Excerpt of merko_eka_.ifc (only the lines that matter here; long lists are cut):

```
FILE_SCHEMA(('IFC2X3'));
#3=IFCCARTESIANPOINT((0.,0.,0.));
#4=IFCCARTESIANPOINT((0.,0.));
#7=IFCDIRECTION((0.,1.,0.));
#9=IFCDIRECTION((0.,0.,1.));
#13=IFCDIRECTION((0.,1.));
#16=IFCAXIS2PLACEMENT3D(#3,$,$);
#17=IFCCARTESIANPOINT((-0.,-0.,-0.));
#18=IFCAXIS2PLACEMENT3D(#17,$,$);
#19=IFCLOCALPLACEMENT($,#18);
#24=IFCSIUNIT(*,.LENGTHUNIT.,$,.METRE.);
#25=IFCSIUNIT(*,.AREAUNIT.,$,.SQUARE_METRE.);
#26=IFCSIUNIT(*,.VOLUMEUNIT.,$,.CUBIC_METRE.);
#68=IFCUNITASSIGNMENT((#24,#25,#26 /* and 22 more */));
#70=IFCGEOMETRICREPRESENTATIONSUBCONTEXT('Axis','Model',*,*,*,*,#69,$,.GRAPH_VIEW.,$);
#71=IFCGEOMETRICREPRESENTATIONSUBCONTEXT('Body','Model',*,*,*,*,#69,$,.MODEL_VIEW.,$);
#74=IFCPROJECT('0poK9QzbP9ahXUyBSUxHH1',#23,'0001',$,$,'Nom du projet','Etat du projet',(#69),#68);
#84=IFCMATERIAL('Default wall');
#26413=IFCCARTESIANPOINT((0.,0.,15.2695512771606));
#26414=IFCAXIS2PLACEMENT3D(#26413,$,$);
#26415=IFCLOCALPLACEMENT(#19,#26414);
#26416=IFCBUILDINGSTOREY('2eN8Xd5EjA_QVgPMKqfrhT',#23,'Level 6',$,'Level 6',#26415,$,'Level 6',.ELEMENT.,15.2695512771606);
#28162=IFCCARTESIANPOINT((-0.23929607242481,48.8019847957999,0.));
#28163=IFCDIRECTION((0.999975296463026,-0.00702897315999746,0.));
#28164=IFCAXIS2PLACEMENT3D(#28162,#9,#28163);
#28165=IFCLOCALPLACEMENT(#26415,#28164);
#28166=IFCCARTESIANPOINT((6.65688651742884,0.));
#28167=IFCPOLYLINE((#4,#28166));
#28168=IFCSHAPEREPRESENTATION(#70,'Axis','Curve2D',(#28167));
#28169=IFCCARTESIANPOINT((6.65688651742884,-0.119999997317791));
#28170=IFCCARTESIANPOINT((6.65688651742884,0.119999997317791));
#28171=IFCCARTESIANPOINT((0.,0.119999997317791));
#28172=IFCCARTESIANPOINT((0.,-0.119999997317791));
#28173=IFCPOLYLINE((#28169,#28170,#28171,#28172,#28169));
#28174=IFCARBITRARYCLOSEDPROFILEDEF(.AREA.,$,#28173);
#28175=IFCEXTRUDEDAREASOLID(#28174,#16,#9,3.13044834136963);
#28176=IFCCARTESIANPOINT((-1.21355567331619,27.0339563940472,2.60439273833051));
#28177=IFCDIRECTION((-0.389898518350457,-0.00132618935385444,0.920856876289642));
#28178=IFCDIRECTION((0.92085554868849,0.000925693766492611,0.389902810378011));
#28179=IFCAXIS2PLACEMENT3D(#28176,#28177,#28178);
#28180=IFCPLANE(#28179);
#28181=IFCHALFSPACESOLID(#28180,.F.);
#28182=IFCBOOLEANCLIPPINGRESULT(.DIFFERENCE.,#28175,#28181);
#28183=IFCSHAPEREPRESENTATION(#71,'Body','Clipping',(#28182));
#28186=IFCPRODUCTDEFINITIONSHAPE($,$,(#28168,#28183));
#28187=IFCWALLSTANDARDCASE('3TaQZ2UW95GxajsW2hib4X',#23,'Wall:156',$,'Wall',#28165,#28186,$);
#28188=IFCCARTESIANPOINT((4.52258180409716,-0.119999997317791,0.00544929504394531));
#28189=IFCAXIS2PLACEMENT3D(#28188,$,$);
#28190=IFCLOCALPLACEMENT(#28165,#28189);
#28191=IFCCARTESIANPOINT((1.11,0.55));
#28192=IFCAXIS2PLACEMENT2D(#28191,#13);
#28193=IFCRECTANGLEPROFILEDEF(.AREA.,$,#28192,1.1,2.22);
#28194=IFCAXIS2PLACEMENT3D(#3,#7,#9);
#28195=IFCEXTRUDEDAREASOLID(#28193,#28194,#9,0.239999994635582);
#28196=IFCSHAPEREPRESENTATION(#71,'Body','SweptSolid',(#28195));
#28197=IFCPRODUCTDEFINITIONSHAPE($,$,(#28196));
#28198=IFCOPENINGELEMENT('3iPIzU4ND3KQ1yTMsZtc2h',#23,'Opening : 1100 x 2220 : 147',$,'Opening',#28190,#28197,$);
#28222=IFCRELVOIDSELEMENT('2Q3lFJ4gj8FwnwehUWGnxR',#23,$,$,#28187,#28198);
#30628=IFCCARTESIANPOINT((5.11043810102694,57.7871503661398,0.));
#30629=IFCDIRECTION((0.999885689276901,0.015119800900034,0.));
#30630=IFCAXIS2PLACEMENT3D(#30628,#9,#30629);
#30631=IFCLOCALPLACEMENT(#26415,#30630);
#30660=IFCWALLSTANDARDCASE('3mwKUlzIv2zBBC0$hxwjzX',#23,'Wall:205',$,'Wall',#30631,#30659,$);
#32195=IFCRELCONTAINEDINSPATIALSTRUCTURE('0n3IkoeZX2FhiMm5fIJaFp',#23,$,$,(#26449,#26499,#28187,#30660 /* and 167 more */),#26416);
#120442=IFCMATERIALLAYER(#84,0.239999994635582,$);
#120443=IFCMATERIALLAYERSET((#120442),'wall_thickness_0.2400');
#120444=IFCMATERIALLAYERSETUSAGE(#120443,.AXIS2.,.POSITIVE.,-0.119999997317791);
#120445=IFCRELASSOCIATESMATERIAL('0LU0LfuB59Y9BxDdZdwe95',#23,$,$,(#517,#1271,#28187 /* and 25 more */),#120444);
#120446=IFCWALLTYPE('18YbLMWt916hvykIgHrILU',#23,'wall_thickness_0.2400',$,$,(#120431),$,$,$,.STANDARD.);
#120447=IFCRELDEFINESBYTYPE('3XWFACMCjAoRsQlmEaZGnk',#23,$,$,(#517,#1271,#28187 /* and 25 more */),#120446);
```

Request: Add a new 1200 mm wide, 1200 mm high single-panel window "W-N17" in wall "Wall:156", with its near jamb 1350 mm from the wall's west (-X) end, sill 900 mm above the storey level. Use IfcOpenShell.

```python
import numpy as np
import ifcopenshell
import ifcopenshell.api.feature
import ifcopenshell.api.geometry
import ifcopenshell.api.root
import ifcopenshell.api.spatial
import ifcopenshell.api.type
import ifcopenshell.geom
import ifcopenshell.util.element
import ifcopenshell.util.placement
import ifcopenshell.util.representation
import ifcopenshell.util.shape
import ifcopenshell.util.unit

model = ifcopenshell.open("merko_eka_.ifc")
unit_scale = ifcopenshell.util.unit.calculate_unit_scale(model)
settings = ifcopenshell.geom.settings()


def volume(element):
    """Net volume in cubic metres, openings subtracted."""
    shape = ifcopenshell.geom.create_shape(settings, element)
    return ifcopenshell.util.shape.get_volume(shape.geometry)


wall = model.by_guid("3TaQZ2UW95GxajsW2hib4X")
storey = ifcopenshell.util.element.get_container(wall, ifc_class="IfcBuildingStorey")
context = ifcopenshell.util.representation.get_context(model, "Model", "Body", "MODEL_VIEW")
before = volume(wall)

width, height, from_end, sill = 1.2, 1.2, 1.35, 0.9  # metres

# The wall runs along its own X axis, and the end named is its -X end.
wall_shape = ifcopenshell.geom.create_shape(settings, wall)
x, y, z = ifcopenshell.util.shape.get_vertices(wall_shape.geometry).T
start = x.min() + from_end
face, thickness = float(y.min()), float(y.max() - y.min())
wall_matrix = ifcopenshell.util.placement.get_local_placement(wall.ObjectPlacement)
level = ifcopenshell.util.placement.get_local_placement(storey.ObjectPlacement)[2, 3]


def in_wall(x, y):
    """Placement at x, y metres in the wall's axes, at sill height."""
    matrix = wall_matrix.copy()
    matrix[:, 3] = wall_matrix @ np.array([x / unit_scale, y / unit_scale, 0.0, 1.0])
    matrix[2, 3] = level + sill / unit_scale
    return matrix


# Opening: a box that overshoots both wall faces by 50 mm.
opening = ifcopenshell.api.root.create_entity(model, ifc_class="IfcOpeningElement")
box = ifcopenshell.api.geometry.add_wall_representation(
    model, context=context, length=width, height=height, thickness=thickness + 0.1
)
ifcopenshell.api.geometry.assign_representation(model, product=opening, representation=box)
ifcopenshell.api.geometry.edit_object_placement(model, product=opening, matrix=in_wall(start, face - 0.05), is_si=False)
ifcopenshell.api.feature.add_feature(model, feature=opening, element=wall)

window = ifcopenshell.api.root.create_entity(model, ifc_class="IfcWindow", name="W-N17")
window.OverallWidth, window.OverallHeight = width / unit_scale, height / unit_scale
body = ifcopenshell.api.geometry.add_window_representation(
    model,
    context=context,
    overall_width=window.OverallWidth,
    overall_height=window.OverallHeight,
    partition_type="SINGLE_PANEL",
)
ifcopenshell.api.geometry.assign_representation(model, product=window, representation=body)
ifcopenshell.api.spatial.assign_container(model, products=[window], relating_structure=storey)
fills = ifcopenshell.api.feature.add_filling(model, opening=opening, element=window)
fills.OwnerHistory = window.OwnerHistory  # required in IFC2X3

# IFC2X3 keeps the operation on the window style.
style = ifcopenshell.api.root.create_entity(model, ifc_class="IfcWindowStyle", name="W-N17")
style.OperationType, style.ConstructionType = "SINGLE_PANEL", "NOTDEFINED"
style.ParameterTakesPrecedence = style.Sizeable = False
ifcopenshell.api.type.assign_type(model, related_objects=[window], relating_type=style)

# Centre the window in the wall's thickness.
ifcopenshell.api.geometry.edit_object_placement(model, product=window, matrix=in_wall(start, face), is_si=False)
window_shape = ifcopenshell.geom.create_shape(settings, window)
depth = ifcopenshell.util.shape.get_vertices(window_shape.geometry)[:, 1]
offset = face + thickness / 2 - (depth.min() + depth.max()) / 2
ifcopenshell.api.geometry.edit_object_placement(model, product=window, matrix=in_wall(start, offset), is_si=False)

after = volume(wall)

print(f"wall volume {before:.3f} -> {after:.3f} m3")

model.write("merko_eka__edited.ifc")
```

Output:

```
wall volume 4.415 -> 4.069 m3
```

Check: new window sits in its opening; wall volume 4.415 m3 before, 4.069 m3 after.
